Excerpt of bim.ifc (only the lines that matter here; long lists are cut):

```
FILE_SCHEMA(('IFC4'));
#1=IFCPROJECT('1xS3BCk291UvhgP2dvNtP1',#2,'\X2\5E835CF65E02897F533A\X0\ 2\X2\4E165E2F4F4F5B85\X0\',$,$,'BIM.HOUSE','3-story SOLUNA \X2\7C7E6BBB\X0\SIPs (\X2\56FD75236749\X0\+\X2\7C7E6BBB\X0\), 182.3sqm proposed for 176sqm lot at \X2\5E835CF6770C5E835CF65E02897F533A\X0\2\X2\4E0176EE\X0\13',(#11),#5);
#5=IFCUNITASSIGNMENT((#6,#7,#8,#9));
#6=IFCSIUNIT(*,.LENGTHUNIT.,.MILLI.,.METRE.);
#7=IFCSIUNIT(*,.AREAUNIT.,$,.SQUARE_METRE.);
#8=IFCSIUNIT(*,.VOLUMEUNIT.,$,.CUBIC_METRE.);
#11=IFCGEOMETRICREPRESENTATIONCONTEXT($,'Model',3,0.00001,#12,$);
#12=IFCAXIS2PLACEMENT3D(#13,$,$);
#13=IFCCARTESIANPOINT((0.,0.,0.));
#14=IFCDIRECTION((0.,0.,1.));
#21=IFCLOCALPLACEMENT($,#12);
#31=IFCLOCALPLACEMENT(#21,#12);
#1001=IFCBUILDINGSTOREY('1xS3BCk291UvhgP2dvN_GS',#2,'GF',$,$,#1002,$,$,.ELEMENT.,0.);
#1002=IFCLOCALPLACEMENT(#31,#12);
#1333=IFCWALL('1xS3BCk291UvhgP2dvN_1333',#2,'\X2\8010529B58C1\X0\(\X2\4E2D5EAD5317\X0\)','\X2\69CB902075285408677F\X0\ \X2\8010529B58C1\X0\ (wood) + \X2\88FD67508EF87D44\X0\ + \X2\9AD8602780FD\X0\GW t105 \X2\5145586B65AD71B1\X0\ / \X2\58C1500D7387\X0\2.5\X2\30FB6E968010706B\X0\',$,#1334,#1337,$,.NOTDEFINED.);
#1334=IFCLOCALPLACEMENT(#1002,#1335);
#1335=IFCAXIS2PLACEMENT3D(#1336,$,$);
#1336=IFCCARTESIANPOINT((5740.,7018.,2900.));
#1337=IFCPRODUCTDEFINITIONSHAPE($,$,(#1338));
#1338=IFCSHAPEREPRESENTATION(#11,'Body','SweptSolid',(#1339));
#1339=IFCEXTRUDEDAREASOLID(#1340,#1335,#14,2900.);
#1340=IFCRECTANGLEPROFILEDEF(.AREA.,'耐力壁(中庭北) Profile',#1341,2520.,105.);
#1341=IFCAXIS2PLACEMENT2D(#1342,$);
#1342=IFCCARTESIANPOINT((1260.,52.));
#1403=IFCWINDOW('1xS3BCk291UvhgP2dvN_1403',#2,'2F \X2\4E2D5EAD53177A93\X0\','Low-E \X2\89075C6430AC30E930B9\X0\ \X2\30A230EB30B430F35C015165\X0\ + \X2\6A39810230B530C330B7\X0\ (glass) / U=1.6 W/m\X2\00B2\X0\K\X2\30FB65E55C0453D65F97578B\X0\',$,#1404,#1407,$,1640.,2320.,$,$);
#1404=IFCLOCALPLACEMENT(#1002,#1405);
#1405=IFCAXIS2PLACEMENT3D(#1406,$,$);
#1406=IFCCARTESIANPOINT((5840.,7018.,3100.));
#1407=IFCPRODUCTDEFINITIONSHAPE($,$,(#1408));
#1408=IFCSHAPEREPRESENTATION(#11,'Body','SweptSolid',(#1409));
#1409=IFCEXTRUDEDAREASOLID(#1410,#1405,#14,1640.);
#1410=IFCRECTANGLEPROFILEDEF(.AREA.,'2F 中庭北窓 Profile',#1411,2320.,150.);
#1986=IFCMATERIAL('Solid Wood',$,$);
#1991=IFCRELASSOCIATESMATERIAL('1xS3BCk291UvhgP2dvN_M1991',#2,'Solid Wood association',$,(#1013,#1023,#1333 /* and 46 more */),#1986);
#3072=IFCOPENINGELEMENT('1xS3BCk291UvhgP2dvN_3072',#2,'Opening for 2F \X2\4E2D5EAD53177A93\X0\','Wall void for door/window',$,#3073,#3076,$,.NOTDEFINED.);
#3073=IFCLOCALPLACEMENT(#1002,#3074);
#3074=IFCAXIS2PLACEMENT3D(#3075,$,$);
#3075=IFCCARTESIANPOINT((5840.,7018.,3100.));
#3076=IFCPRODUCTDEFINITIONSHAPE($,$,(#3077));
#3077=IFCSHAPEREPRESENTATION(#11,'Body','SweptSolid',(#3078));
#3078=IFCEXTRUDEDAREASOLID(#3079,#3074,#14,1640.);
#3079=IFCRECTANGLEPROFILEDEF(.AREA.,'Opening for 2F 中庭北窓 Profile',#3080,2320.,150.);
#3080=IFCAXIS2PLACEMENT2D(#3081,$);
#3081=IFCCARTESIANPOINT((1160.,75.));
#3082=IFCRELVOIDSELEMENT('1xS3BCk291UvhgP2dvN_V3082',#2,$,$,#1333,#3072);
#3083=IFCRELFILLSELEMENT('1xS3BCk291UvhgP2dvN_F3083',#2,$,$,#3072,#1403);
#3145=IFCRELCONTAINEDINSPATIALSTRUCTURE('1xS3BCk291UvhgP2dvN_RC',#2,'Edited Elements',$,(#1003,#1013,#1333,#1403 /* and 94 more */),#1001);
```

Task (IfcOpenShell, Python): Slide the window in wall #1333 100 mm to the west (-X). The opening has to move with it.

```python
import ifcopenshell
import ifcopenshell.api.geometry
import ifcopenshell.util.placement

model = ifcopenshell.open("bim.ifc")

window = model.by_guid("1xS3BCk291UvhgP2dvN_1403")
opening = window.FillsVoids[0].RelatingOpeningElement
wall = opening.VoidsElements[0].RelatingBuildingElement

wall_matrix = ifcopenshell.util.placement.get_local_placement(wall.ObjectPlacement)
shift = wall_matrix[:3, 0] * -100.0
before = ifcopenshell.util.placement.get_local_placement(window.ObjectPlacement)[:3, 3].copy()

# The window is not placed relative to its opening, so move both.
for product in (opening, window):
    matrix = ifcopenshell.util.placement.get_local_placement(product.ObjectPlacement)
    matrix[:3, 3] += shift
    ifcopenshell.api.geometry.edit_object_placement(model, product=product, matrix=matrix, is_si=False)

after = ifcopenshell.util.placement.get_local_placement(window.ObjectPlacement)[:3, 3]
print("window moved by", (after - before).round(3) + 0.0)

model.write("bim-out.ifc")
```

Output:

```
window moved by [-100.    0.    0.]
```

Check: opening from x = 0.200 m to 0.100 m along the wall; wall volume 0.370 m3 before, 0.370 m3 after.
